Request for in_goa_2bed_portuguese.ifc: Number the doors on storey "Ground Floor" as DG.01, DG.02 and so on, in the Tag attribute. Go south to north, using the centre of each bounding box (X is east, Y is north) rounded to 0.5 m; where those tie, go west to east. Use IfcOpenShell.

First a look at what the model holds.

```python
import ifcopenshell
import ifcopenshell.util.element
import ifcopenshell.util.placement

model = ifcopenshell.open("in_goa_2bed_portuguese.ifc")
print(model.schema)
storey = next(s for s in model.by_type("IfcBuildingStorey") if s.Name == "Ground Floor")
doors = [e for e in ifcopenshell.util.element.get_decomposition(storey) if e.is_a("IfcDoor")]
for e in sorted(doors, key=lambda e: e.id()):
    origin = ifcopenshell.util.placement.get_local_placement(e.ObjectPlacement)[:3, 3]
    print(e.id(), e.Tag, e.Name, origin.round(2) + 0.0, sep=" | ")
```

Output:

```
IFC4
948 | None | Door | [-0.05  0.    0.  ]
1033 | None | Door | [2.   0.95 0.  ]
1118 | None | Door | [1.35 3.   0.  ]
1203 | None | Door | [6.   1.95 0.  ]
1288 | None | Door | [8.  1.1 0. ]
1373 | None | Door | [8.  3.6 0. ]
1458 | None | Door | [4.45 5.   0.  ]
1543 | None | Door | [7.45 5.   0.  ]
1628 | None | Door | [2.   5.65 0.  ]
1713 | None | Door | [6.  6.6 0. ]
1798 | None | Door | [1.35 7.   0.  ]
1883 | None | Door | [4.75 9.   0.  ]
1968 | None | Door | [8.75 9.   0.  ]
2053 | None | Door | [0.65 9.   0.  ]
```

```python
import ifcopenshell
import ifcopenshell.geom
import ifcopenshell.util.element
import ifcopenshell.util.shape

model = ifcopenshell.open("in_goa_2bed_portuguese.ifc")
settings = ifcopenshell.geom.settings()
settings.set("use-world-coords", True)


def centre(element):
    shape = ifcopenshell.geom.create_shape(settings, element)
    return ifcopenshell.util.shape.get_bbox_centroid(shape.geometry)


storey = next(s for s in model.by_type("IfcBuildingStorey") if s.Name == "Ground Floor")
doors = [e for e in ifcopenshell.util.element.get_decomposition(storey) if e.is_a("IfcDoor")]

# Insertion points can sit at a corner or the storey origin, so sort by the geometry (in metres).
centres = {e: centre(e) for e in doors}
doors.sort(key=lambda e: (round(centres[e][1] / 0.5), centres[e][0]))

for i, e in enumerate(doors, start=1):
    number = f"DG.{i:02d}"
    e.Tag = number
    print(e.id(), number)

model.write("in_goa_2bed_portuguese-out.ifc")
```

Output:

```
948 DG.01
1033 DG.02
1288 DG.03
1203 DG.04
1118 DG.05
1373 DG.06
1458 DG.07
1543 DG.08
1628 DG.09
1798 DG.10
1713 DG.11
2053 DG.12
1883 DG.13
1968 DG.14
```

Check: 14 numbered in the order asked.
